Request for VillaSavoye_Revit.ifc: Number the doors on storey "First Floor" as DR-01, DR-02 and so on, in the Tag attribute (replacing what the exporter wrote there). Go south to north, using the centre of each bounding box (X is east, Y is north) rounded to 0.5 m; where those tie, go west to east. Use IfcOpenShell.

First a look at what the model holds.

```python
import ifcopenshell
import ifcopenshell.util.element
import ifcopenshell.util.placement

model = ifcopenshell.open("VillaSavoye_Revit.ifc")
print(model.schema)
storey = next(s for s in model.by_type("IfcBuildingStorey") if s.Name == "First Floor")
doors = [e for e in ifcopenshell.util.element.get_decomposition(storey) if e.is_a("IfcDoor")]
for e in sorted(doors, key=lambda e: e.id()):
    origin = ifcopenshell.util.placement.get_local_placement(e.ObjectPlacement)[:3, 3]
    print(e.id(), e.Tag, e.Name, origin.round(2) + 0.0, sep=" | ")
```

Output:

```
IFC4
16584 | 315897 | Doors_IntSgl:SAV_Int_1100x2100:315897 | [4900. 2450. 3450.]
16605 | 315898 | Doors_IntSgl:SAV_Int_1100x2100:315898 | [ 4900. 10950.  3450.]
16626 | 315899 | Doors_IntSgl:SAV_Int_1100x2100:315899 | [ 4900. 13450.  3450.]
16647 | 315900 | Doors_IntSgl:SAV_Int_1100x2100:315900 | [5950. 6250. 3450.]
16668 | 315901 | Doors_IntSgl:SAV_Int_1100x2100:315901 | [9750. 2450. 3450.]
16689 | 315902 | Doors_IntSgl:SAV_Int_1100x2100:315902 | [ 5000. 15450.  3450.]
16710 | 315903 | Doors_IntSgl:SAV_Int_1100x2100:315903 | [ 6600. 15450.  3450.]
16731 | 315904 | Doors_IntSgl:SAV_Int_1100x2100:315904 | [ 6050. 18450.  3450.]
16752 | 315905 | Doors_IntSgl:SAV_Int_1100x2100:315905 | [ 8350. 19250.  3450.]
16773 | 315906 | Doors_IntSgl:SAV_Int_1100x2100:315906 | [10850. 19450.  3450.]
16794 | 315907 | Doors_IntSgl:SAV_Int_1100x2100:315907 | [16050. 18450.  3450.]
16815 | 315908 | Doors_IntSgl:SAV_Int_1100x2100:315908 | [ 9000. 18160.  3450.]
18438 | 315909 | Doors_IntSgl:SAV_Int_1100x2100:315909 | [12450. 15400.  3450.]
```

```python
import ifcopenshell
import ifcopenshell.geom
import ifcopenshell.util.element
import ifcopenshell.util.shape

model = ifcopenshell.open("VillaSavoye_Revit.ifc")
settings = ifcopenshell.geom.settings()
settings.set("use-world-coords", True)


def centre(element):
    shape = ifcopenshell.geom.create_shape(settings, element)
    return ifcopenshell.util.shape.get_bbox_centroid(shape.geometry)


storey = next(s for s in model.by_type("IfcBuildingStorey") if s.Name == "First Floor")
doors = [e for e in ifcopenshell.util.element.get_decomposition(storey) if e.is_a("IfcDoor")]

# Insertion points can sit at a corner or the storey origin, so sort by the geometry (in metres).
centres = {e: centre(e) for e in doors}
doors.sort(key=lambda e: (round(centres[e][1] / 0.5), centres[e][0]))

for i, e in enumerate(doors, start=1):
    number = f"DR-{i:02d}"
    e.Tag = number
    print(e.id(), number)

model.write("VillaSavoye_Revit_v2.ifc")
```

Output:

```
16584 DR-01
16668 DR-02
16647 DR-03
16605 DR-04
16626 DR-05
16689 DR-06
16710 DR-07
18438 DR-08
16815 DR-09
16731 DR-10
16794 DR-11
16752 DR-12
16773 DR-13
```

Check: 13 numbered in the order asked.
